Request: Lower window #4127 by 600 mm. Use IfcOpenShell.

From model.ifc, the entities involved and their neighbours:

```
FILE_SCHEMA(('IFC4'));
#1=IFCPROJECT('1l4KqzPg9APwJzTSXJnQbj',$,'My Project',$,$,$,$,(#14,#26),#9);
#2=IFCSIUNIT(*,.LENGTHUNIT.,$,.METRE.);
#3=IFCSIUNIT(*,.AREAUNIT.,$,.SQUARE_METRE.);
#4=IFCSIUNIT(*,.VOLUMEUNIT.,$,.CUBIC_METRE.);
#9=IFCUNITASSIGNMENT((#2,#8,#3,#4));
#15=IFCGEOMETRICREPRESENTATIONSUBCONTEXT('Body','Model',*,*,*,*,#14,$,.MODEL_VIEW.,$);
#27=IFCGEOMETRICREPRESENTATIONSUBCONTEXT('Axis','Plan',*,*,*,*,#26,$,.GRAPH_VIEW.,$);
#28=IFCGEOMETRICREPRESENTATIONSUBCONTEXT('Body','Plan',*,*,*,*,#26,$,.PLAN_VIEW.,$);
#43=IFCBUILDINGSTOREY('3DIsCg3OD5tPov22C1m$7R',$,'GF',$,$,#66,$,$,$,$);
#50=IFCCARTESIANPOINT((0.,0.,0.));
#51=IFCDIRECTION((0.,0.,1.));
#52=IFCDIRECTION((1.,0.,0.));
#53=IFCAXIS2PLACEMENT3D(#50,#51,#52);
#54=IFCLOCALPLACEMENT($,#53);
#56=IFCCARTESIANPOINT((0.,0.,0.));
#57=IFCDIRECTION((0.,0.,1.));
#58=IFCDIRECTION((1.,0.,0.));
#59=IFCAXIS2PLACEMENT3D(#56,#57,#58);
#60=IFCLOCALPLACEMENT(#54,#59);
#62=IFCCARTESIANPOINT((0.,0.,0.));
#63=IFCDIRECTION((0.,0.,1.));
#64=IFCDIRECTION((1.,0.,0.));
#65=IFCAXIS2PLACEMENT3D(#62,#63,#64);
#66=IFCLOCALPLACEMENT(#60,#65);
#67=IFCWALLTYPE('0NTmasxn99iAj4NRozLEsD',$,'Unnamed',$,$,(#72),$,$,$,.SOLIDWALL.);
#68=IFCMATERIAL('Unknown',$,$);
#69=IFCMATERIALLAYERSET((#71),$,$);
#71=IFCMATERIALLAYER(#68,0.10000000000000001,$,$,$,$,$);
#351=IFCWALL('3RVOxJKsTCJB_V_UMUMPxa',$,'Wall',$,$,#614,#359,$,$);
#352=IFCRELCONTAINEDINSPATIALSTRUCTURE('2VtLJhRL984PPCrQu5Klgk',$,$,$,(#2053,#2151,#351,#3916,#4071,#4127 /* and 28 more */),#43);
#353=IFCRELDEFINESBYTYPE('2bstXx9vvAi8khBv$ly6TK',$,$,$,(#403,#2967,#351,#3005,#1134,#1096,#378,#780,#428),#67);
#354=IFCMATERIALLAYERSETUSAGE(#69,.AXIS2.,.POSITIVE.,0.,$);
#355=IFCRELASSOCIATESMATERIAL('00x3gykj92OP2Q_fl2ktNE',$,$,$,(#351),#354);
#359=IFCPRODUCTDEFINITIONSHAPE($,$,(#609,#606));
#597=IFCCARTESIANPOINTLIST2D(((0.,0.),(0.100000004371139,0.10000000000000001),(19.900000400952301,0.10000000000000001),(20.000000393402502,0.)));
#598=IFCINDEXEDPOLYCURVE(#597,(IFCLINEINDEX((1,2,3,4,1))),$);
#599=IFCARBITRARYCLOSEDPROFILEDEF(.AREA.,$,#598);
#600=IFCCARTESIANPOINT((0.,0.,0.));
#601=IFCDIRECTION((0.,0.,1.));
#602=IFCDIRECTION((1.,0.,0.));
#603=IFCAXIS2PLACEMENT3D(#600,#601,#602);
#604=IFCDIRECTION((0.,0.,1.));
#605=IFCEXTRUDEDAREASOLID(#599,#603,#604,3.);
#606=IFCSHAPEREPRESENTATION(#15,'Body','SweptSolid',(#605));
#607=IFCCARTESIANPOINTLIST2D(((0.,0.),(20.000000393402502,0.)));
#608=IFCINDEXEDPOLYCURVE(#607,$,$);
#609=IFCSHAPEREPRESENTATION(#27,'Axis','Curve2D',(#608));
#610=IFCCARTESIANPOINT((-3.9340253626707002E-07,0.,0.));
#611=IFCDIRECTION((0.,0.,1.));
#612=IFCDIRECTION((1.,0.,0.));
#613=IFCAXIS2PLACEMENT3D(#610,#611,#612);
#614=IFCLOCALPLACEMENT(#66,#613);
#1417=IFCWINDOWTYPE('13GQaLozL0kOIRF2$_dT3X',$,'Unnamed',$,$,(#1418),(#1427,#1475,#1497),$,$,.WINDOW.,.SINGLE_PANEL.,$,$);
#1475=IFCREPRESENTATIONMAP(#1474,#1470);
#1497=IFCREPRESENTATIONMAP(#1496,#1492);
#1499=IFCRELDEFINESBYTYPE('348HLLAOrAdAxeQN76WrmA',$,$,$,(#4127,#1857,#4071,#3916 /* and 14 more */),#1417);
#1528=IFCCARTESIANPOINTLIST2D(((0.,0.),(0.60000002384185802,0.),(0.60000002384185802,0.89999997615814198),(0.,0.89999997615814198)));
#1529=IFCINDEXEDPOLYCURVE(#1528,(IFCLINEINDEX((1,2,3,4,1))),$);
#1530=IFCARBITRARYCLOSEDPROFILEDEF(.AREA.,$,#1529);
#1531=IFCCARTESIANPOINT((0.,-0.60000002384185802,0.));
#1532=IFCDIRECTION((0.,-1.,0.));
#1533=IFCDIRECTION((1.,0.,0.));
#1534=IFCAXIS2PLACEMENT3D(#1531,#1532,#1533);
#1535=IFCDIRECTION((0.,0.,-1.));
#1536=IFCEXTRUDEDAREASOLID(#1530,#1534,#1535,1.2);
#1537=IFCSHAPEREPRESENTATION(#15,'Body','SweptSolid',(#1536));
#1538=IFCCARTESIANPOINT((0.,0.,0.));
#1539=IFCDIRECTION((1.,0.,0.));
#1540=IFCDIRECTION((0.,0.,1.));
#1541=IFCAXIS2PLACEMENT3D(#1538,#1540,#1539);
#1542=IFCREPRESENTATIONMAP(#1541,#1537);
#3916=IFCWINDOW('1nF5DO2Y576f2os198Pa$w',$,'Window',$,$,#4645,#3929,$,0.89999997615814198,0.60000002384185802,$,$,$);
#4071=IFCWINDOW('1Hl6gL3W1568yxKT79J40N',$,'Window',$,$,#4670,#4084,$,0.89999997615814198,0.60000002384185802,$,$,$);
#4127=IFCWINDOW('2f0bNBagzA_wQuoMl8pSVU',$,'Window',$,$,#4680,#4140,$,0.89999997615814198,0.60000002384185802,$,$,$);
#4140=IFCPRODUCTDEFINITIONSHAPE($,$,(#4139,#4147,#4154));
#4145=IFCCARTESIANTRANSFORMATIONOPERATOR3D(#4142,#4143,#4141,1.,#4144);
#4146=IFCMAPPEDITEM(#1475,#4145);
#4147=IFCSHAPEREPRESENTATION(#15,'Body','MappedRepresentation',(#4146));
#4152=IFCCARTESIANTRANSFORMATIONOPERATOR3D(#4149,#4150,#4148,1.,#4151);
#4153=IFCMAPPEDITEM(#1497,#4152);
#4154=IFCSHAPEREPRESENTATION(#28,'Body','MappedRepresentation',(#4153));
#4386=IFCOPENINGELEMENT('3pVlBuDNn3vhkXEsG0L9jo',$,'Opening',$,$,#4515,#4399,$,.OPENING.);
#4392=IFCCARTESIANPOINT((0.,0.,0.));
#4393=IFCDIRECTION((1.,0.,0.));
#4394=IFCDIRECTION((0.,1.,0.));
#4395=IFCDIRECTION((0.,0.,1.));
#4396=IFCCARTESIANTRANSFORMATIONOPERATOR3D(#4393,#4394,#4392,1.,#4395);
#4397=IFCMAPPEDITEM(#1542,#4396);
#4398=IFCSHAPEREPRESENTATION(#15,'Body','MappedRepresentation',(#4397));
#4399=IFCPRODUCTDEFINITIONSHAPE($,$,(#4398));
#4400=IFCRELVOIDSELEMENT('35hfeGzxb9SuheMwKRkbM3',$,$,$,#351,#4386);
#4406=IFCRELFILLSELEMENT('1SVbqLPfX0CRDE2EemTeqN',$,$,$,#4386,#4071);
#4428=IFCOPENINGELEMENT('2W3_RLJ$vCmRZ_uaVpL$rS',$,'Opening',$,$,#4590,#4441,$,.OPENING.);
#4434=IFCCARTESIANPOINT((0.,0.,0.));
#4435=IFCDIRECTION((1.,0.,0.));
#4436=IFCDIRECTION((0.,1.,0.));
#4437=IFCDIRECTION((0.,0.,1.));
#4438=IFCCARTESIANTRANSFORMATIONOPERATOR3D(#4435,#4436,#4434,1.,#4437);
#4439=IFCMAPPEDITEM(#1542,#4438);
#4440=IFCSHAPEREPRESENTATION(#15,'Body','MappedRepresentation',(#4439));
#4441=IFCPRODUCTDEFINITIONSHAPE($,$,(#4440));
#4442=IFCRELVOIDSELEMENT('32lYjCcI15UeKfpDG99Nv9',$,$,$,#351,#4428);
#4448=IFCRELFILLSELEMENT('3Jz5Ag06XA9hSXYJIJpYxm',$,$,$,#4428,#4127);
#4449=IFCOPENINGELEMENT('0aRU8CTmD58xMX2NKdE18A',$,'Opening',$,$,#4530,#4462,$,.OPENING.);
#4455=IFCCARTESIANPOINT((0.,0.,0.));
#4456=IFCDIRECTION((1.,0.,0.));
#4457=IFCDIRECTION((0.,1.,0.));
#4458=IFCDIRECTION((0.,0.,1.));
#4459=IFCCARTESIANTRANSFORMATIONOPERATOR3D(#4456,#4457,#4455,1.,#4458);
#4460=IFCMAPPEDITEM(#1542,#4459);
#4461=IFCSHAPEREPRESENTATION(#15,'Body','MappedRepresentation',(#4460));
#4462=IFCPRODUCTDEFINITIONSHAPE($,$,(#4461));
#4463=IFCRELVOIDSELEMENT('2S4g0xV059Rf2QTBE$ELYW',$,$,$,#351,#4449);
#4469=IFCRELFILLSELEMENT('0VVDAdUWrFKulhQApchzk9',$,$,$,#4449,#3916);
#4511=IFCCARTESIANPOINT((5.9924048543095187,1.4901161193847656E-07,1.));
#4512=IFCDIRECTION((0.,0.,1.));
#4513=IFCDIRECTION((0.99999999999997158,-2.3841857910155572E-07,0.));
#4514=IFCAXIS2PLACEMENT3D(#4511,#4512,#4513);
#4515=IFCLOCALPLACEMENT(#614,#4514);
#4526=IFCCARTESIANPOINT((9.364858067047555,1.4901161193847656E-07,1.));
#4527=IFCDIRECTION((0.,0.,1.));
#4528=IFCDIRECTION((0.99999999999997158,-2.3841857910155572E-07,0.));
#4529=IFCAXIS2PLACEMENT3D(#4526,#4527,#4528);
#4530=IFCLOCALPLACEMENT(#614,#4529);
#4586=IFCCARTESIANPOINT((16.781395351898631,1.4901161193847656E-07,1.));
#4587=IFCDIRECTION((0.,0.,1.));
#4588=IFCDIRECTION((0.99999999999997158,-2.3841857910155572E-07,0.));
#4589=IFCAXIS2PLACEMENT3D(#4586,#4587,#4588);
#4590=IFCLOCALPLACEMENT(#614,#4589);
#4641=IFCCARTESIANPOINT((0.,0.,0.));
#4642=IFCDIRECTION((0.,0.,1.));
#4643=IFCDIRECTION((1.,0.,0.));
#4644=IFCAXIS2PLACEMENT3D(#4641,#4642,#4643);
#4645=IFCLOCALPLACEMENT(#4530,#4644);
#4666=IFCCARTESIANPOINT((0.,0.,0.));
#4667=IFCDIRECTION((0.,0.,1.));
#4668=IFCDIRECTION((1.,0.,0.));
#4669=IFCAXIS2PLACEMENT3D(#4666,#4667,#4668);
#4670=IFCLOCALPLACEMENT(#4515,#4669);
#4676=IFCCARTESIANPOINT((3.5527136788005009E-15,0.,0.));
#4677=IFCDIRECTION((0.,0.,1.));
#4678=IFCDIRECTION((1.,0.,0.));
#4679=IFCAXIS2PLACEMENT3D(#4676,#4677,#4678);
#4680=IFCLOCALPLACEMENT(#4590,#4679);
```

```python
import numpy as np
import ifcopenshell
import ifcopenshell.api.geometry
import ifcopenshell.util.placement
import ifcopenshell.util.unit

model = ifcopenshell.open("model.ifc")
unit_scale = ifcopenshell.util.unit.calculate_unit_scale(model)

window = model.by_id(4127)
opening = window.FillsVoids[0].RelatingOpeningElement
dz = -0.6 / unit_scale

shift = np.array([0.0, 0.0, dz])
# The window is placed relative to its opening, so it follows when the opening moves.
matrix = ifcopenshell.util.placement.get_local_placement(opening.ObjectPlacement)
matrix[:3, 3] += shift
ifcopenshell.api.geometry.edit_object_placement(
    model, product=opening, matrix=matrix, is_si=False, should_transform_children=True
)

print(f"moved by {dz * unit_scale:+.3f} m")

model.write("model_rev.ifc")
```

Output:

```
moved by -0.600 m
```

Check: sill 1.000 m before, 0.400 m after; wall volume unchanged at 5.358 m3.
